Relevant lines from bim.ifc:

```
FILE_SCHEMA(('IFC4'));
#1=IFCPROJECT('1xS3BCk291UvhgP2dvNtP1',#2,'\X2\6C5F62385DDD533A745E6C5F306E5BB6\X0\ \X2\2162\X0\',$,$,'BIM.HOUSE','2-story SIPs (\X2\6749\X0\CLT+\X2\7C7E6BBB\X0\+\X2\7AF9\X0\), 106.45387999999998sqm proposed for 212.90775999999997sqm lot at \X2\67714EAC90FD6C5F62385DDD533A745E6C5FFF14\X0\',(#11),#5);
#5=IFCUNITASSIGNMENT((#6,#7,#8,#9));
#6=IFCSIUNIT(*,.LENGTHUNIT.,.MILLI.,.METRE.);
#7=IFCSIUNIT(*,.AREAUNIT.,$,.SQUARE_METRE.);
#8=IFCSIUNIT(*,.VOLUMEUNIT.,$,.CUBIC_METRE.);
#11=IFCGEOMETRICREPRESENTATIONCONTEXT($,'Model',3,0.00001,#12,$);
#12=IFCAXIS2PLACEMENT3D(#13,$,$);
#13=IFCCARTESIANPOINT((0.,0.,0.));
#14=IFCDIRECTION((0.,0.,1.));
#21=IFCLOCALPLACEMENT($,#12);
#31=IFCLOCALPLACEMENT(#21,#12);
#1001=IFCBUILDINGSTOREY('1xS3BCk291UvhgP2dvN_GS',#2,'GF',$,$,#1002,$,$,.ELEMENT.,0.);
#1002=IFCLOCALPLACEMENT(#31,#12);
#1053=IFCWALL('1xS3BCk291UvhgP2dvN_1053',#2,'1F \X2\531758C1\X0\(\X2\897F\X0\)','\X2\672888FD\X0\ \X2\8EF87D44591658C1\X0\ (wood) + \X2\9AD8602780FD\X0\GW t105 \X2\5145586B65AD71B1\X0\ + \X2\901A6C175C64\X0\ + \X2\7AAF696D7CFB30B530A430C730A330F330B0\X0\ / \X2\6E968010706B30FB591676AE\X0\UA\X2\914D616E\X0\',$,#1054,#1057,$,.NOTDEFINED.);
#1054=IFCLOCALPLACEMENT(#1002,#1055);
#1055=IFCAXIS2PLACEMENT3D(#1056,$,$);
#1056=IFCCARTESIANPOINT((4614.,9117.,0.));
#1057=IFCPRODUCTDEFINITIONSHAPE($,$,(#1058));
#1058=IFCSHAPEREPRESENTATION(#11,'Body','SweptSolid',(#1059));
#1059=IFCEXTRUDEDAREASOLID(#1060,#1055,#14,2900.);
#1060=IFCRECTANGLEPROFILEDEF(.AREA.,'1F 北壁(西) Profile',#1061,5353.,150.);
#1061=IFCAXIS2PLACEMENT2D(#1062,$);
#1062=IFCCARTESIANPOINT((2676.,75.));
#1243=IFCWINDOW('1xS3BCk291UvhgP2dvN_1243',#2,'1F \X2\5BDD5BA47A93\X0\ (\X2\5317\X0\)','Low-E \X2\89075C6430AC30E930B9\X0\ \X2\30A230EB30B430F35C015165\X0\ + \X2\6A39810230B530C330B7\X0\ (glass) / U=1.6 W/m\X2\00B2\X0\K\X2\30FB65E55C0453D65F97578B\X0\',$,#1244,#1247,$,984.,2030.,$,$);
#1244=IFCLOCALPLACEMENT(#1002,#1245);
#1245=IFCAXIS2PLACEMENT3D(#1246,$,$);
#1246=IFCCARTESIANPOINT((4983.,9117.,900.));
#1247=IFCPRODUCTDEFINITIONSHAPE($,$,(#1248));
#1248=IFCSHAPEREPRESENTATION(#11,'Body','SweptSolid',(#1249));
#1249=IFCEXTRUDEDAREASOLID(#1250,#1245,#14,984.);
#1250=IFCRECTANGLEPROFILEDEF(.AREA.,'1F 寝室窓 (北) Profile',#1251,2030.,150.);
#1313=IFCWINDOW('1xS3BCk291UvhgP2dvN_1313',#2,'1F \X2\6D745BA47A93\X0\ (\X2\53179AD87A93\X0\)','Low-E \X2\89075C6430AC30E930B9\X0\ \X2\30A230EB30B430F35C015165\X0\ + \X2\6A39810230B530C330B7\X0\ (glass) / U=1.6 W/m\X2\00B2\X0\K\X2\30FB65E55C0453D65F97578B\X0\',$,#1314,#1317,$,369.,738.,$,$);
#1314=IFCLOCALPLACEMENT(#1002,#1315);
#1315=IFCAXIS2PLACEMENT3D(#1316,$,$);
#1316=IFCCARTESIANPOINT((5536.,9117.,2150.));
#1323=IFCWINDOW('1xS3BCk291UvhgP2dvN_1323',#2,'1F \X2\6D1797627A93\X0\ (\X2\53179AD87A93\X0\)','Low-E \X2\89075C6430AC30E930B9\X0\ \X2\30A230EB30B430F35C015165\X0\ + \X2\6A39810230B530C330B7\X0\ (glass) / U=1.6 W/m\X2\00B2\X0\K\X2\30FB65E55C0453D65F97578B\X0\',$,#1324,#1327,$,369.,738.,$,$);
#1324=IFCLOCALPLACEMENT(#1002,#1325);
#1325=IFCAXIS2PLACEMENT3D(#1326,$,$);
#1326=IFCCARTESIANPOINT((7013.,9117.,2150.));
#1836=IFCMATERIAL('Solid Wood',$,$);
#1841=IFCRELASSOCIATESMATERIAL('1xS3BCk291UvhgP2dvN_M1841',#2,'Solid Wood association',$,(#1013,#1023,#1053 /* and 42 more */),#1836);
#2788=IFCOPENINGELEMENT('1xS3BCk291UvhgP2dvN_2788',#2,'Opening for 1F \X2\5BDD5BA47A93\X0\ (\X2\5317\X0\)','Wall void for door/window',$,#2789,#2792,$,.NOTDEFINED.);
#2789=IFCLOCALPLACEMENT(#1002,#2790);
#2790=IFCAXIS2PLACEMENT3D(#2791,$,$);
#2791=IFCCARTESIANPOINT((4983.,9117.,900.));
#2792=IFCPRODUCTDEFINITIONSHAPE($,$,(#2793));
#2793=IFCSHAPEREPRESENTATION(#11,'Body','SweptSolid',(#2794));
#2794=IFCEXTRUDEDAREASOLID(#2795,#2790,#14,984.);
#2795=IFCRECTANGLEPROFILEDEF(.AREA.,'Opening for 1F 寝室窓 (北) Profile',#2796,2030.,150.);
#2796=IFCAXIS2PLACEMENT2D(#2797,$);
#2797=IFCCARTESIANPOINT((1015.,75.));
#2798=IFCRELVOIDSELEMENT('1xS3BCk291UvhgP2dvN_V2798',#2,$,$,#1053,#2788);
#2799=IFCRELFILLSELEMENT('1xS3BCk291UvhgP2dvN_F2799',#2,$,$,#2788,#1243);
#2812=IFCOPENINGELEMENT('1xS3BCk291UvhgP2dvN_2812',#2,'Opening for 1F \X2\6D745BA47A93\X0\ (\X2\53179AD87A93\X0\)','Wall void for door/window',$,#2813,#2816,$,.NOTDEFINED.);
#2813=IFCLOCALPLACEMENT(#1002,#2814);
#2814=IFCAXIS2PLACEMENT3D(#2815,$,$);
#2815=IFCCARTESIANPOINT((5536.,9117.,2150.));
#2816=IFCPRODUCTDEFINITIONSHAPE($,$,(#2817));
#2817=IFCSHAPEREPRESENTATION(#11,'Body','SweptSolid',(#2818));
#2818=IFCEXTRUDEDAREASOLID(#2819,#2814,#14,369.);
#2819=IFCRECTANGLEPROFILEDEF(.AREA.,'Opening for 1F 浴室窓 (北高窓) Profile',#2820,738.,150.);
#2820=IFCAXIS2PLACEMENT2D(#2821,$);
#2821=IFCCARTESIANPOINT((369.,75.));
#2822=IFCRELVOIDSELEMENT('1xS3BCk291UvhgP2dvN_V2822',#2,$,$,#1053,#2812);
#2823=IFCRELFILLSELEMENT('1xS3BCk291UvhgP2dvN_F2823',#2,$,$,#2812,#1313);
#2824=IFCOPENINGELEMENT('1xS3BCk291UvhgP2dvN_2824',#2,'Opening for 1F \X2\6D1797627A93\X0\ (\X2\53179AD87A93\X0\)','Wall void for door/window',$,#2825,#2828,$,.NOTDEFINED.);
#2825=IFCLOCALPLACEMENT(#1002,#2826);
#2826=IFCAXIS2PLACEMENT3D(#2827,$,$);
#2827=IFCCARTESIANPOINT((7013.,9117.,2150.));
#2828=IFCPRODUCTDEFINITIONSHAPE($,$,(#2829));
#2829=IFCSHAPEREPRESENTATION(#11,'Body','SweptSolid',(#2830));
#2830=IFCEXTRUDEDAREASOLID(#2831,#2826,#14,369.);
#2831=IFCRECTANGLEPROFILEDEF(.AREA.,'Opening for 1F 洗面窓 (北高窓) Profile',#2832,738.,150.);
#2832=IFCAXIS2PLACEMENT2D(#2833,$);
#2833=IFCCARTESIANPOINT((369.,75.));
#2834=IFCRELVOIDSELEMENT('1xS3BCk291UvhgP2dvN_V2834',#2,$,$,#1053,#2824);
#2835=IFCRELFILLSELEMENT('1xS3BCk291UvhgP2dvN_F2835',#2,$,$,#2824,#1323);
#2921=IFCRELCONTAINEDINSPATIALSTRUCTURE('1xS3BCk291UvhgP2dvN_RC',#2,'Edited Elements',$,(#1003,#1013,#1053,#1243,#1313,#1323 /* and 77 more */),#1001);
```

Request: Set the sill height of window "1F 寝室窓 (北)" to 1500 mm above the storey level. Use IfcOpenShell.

```python
import numpy as np
import ifcopenshell
import ifcopenshell.api.geometry
import ifcopenshell.geom
import ifcopenshell.util.element
import ifcopenshell.util.placement
import ifcopenshell.util.shape
import ifcopenshell.util.unit

model = ifcopenshell.open("bim.ifc")
unit_scale = ifcopenshell.util.unit.calculate_unit_scale(model)

window = model.by_guid("1xS3BCk291UvhgP2dvN_1243")
opening = window.FillsVoids[0].RelatingOpeningElement
storey = ifcopenshell.util.element.get_container(window, ifc_class="IfcBuildingStorey")
level = ifcopenshell.util.placement.get_local_placement(storey.ObjectPlacement)[2, 3]

# The opening's origin need not be at the sill, so measure its lowest point.
shape = ifcopenshell.geom.create_shape(ifcopenshell.geom.settings(), opening)
bottom = ifcopenshell.util.shape.get_shape_bottom_elevation(shape, shape.geometry) / unit_scale
dz = level + 1500.0 - bottom

shift = np.array([0.0, 0.0, dz])
# The window is not placed relative to its opening, so move both.
for product in (opening, window):
    matrix = ifcopenshell.util.placement.get_local_placement(product.ObjectPlacement)
    matrix[:3, 3] += shift
    ifcopenshell.api.geometry.edit_object_placement(model, product=product, matrix=matrix, is_si=False)

print(f"moved by {dz * unit_scale:+.3f} m")

model.write("bim_v2.ifc")
```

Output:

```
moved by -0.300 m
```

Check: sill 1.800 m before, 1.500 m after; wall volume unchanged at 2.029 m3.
